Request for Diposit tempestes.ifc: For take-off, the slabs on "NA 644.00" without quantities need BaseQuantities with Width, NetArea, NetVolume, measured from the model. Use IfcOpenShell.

First a look at what the model holds.

```python
import ifcopenshell
import ifcopenshell.util.element
import ifcopenshell.util.unit

model = ifcopenshell.open("Diposit tempestes.ifc")
print(model.schema)
for unit_type in ("LENGTHUNIT", "AREAUNIT", "VOLUMEUNIT"):
    print(unit_type, ifcopenshell.util.unit.calculate_unit_scale(model, unit_type))
storey = next(s for s in model.by_type("IfcBuildingStorey") if s.Name == "NA 644.00")
slabs = [e for e in ifcopenshell.util.element.get_decomposition(storey) if e.is_a("IfcSlab")]
for e in sorted(slabs, key=lambda e: e.id()):
    print(e.id(), e.is_a(), e.Name, list(ifcopenshell.util.element.get_psets(e, qtos_only=True)), sep=" | ")
```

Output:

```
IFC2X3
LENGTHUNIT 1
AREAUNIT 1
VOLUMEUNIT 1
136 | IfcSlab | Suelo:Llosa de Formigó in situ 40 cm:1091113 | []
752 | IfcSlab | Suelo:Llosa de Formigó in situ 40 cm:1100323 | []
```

```python
import ifcopenshell
import ifcopenshell.api.pset
import ifcopenshell.geom
import ifcopenshell.util.element
import ifcopenshell.util.shape
import ifcopenshell.util.unit

model = ifcopenshell.open("Diposit tempestes.ifc")
unit_scale = ifcopenshell.util.unit.calculate_unit_scale(model)
area_scale = ifcopenshell.util.unit.calculate_unit_scale(model, "AREAUNIT")
volume_scale = ifcopenshell.util.unit.calculate_unit_scale(model, "VOLUMEUNIT")
settings = ifcopenshell.geom.settings()

storey = next(s for s in model.by_type("IfcBuildingStorey") if s.Name == "NA 644.00")
slabs = [e for e in ifcopenshell.util.element.get_decomposition(storey) if e.is_a("IfcSlab")]

for e in sorted(slabs, key=lambda e: e.id()):
    if ifcopenshell.util.element.get_psets(e, qtos_only=True, should_inherit=False):
        continue
    # Geometry comes back in metres, in the element's own axes.
    shape = ifcopenshell.geom.create_shape(settings, e)
    values = {
        "Width": ifcopenshell.util.shape.get_z(shape.geometry) / unit_scale,
        "NetArea": ifcopenshell.util.shape.get_footprint_area(shape.geometry) / area_scale,
        "NetVolume": ifcopenshell.util.shape.get_volume(shape.geometry) / volume_scale,
    }
    qto = ifcopenshell.api.pset.add_qto(model, product=e, name="BaseQuantities")
    ifcopenshell.api.pset.edit_qto(model, qto=qto, properties=values)
    print(e.id(), {k: round(v, 3) for k, v in values.items()})

model.write("Diposit tempestes_rev.ifc")
```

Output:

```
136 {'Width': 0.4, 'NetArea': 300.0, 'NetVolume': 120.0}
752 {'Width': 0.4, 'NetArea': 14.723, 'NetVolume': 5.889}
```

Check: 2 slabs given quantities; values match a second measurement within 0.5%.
